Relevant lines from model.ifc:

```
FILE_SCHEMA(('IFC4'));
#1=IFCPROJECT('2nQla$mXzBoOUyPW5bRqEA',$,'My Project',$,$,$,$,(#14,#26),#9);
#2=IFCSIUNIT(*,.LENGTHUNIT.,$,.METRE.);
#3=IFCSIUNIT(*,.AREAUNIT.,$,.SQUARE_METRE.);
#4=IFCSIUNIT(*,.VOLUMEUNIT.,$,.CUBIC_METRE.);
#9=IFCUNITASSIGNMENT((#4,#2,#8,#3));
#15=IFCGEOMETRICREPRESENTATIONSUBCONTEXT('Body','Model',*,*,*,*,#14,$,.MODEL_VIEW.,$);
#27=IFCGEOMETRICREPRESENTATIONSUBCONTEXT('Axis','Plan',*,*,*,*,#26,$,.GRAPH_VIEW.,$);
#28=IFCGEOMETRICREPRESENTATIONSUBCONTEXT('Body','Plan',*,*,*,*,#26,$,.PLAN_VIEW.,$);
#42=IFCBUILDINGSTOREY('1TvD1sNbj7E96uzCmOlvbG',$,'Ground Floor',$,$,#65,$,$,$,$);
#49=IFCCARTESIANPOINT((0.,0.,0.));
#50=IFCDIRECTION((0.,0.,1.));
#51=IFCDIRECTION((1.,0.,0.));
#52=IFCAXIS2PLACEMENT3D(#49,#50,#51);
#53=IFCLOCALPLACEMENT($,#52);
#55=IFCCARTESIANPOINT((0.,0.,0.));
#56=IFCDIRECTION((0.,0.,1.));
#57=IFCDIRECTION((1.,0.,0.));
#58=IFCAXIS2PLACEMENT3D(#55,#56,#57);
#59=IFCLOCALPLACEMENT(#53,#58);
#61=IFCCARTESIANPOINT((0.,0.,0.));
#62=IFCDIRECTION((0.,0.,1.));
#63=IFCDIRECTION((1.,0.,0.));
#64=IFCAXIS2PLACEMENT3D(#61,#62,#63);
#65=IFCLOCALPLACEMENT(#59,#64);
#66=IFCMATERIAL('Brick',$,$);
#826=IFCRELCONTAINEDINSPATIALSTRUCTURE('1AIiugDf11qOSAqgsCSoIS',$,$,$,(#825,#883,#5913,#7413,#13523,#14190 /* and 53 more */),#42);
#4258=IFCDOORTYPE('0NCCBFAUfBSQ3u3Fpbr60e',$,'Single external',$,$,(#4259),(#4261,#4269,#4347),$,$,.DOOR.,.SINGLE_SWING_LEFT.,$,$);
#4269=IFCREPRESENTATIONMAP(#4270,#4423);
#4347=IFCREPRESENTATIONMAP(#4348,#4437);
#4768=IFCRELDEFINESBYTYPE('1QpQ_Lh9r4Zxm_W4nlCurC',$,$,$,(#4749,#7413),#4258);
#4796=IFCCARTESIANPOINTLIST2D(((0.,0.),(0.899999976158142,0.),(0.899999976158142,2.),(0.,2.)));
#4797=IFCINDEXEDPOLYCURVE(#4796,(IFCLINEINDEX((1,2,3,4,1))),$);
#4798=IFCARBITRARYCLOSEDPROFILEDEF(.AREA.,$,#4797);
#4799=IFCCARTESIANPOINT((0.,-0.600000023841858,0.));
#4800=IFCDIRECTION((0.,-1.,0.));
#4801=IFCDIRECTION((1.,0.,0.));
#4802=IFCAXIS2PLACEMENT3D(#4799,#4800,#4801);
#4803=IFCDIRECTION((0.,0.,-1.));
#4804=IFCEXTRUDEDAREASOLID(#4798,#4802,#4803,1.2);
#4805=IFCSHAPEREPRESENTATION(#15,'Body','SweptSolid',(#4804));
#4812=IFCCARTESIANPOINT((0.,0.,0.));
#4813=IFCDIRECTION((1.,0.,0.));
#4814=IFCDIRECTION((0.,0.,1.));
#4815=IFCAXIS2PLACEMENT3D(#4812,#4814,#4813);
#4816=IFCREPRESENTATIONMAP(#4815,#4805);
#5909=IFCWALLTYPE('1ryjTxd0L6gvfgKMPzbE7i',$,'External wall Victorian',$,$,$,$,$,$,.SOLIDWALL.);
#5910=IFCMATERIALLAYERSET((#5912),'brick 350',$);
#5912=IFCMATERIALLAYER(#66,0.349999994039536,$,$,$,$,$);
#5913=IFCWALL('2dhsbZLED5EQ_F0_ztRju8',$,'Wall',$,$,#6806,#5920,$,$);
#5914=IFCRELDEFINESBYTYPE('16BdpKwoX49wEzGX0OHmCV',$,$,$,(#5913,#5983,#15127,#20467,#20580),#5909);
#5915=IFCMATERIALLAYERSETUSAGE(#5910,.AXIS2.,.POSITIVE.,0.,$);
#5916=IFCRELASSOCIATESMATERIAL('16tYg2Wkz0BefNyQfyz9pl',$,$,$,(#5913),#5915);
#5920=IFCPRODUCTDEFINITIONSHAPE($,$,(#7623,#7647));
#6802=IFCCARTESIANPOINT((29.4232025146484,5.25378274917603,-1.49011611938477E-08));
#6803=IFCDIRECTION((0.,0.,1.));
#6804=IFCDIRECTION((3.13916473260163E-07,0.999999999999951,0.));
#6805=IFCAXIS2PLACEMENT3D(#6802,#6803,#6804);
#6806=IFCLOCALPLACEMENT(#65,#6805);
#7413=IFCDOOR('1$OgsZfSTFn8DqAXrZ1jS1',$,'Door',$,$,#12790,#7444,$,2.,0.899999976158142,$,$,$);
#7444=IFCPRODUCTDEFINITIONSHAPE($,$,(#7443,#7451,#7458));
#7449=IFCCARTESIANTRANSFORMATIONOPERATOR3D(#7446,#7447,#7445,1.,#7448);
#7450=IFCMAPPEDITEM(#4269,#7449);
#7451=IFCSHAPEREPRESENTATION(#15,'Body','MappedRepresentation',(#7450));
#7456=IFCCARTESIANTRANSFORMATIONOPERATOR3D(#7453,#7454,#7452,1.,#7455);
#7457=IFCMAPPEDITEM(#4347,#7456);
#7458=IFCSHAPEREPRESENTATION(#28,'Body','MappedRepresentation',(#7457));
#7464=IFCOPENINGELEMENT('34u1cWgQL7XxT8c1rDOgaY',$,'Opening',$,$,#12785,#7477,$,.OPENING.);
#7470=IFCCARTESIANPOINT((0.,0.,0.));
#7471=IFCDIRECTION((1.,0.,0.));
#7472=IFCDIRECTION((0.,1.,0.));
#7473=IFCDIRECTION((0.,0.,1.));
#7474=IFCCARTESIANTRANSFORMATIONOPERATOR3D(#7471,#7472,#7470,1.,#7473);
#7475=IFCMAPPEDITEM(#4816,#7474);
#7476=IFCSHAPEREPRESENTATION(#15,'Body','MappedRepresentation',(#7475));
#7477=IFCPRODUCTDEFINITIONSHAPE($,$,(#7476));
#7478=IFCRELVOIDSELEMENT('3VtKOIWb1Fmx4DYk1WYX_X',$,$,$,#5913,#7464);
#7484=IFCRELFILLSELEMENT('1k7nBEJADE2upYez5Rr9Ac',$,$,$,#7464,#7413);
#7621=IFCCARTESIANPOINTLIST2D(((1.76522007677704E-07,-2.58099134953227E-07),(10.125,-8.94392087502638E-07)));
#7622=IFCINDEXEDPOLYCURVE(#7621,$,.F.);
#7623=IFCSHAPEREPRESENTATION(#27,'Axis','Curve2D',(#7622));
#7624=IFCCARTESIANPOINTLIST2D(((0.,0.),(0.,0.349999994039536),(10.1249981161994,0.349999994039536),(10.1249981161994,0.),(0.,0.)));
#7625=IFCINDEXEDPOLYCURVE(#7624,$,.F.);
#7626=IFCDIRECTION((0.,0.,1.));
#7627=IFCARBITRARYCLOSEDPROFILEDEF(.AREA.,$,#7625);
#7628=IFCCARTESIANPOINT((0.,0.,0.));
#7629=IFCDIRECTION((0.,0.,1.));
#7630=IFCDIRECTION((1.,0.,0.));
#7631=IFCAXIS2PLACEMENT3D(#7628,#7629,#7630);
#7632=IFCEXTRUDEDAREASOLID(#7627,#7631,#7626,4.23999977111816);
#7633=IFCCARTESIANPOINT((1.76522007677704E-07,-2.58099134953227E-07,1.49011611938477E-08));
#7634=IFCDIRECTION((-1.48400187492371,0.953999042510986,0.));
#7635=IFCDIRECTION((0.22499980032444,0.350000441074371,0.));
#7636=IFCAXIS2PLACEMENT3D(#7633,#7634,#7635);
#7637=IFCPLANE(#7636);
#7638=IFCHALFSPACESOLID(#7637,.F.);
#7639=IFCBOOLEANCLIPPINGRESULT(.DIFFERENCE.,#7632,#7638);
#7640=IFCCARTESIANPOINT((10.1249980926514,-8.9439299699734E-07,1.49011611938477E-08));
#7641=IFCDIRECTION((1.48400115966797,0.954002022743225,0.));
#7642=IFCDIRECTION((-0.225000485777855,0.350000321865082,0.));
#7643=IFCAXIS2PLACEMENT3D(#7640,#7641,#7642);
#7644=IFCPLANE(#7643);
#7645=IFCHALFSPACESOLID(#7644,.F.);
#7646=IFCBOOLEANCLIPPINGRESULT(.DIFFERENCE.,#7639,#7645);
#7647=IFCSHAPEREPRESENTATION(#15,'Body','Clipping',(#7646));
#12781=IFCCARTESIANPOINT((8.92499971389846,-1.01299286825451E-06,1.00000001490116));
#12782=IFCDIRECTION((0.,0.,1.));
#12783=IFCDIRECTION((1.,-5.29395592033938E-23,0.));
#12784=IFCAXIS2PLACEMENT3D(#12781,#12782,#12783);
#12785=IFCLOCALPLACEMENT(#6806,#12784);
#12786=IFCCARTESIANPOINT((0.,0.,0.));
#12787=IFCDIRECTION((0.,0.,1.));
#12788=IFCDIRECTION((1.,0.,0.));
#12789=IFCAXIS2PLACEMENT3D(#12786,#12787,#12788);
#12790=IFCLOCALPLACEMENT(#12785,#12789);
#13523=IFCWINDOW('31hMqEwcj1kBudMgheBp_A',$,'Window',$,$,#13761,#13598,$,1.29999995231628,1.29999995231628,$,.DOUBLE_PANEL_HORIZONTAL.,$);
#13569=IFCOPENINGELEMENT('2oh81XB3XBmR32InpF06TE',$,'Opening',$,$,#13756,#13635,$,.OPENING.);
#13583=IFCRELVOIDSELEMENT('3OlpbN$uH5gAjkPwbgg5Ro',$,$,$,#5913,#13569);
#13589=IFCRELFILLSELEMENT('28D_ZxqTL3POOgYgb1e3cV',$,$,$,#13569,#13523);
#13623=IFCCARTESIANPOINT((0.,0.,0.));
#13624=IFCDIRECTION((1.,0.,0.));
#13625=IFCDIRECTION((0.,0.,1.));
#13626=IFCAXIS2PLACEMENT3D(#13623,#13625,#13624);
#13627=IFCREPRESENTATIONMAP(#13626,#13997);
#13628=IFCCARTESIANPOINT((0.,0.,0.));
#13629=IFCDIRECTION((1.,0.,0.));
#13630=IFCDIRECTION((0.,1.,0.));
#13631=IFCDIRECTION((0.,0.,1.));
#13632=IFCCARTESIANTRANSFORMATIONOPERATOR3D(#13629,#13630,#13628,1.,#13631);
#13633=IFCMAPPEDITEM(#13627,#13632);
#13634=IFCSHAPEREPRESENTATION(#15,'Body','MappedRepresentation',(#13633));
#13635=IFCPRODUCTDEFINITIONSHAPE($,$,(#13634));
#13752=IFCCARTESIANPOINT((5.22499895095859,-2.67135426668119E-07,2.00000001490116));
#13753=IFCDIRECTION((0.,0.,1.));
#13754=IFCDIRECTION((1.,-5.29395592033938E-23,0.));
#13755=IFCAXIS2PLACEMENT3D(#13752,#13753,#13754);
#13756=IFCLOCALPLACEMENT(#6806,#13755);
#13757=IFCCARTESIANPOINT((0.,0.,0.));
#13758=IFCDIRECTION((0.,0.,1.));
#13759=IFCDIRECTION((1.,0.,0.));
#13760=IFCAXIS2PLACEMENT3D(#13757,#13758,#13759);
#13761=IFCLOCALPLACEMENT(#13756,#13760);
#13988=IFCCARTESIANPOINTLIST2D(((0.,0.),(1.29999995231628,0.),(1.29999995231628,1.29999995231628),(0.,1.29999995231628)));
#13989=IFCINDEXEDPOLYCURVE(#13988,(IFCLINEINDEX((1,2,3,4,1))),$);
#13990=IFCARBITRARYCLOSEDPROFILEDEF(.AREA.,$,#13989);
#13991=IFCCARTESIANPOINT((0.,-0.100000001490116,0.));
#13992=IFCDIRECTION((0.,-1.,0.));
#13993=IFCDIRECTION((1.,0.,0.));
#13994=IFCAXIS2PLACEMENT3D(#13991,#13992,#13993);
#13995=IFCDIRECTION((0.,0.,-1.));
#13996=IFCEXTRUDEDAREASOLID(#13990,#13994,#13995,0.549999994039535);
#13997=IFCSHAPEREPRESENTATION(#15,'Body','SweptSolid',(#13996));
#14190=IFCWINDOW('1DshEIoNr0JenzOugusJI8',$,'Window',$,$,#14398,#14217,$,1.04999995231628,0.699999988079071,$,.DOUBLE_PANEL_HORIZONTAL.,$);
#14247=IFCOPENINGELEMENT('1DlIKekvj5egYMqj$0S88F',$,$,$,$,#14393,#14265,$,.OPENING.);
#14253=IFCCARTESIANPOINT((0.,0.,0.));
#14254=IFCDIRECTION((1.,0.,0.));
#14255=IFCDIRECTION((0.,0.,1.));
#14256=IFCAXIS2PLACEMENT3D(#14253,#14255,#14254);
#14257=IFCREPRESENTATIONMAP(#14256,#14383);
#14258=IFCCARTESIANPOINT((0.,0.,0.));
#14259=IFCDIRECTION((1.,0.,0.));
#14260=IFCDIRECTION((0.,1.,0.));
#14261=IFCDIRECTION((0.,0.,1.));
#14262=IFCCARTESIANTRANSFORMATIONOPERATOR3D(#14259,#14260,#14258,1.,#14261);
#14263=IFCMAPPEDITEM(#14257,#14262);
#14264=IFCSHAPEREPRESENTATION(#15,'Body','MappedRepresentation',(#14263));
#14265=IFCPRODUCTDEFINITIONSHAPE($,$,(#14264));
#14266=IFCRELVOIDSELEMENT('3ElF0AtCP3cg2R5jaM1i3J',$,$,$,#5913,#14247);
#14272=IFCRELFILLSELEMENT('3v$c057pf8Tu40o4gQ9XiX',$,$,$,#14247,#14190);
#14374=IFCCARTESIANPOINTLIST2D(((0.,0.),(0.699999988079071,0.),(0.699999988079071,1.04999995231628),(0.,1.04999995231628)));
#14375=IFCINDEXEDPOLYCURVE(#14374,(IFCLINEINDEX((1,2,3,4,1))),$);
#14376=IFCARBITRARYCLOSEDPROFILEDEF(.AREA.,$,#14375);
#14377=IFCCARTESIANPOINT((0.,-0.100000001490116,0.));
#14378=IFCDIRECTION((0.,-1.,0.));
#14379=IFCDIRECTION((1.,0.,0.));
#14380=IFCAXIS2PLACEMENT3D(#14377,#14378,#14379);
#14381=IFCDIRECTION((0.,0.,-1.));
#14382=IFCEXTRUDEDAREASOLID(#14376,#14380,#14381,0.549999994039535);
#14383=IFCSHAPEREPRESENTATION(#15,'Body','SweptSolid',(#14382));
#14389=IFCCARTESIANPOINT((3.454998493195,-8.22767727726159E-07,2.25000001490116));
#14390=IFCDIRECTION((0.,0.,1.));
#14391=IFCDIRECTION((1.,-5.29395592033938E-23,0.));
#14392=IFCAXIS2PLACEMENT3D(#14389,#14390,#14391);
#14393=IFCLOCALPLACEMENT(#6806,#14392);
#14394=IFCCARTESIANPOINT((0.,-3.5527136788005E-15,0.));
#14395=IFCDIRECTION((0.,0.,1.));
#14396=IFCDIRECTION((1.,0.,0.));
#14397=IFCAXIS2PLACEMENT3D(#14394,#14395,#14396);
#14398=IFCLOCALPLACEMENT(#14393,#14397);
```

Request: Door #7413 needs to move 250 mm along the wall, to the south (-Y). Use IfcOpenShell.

```python
import ifcopenshell
import ifcopenshell.api.geometry
import ifcopenshell.util.placement
import ifcopenshell.util.unit

model = ifcopenshell.open("model.ifc")
unit_scale = ifcopenshell.util.unit.calculate_unit_scale(model)

door = model.by_guid("1$OgsZfSTFn8DqAXrZ1jS1")
opening = door.FillsVoids[0].RelatingOpeningElement
wall = opening.VoidsElements[0].RelatingBuildingElement

wall_matrix = ifcopenshell.util.placement.get_local_placement(wall.ObjectPlacement)
shift = wall_matrix[:3, 0] * -0.25 / unit_scale
before = ifcopenshell.util.placement.get_local_placement(door.ObjectPlacement)[:3, 3].copy()

# The door is placed relative to its opening, so it follows when the opening moves.
matrix = ifcopenshell.util.placement.get_local_placement(opening.ObjectPlacement)
matrix[:3, 3] += shift
ifcopenshell.api.geometry.edit_object_placement(
    model, product=opening, matrix=matrix, is_si=False, should_transform_children=True
)

after = ifcopenshell.util.placement.get_local_placement(door.ObjectPlacement)[:3, 3]
print("door moved by", (after - before).round(3) + 0.0)

model.write("model_v2.ifc")
```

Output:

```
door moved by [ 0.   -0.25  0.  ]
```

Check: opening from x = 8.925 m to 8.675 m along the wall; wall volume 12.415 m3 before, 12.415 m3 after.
